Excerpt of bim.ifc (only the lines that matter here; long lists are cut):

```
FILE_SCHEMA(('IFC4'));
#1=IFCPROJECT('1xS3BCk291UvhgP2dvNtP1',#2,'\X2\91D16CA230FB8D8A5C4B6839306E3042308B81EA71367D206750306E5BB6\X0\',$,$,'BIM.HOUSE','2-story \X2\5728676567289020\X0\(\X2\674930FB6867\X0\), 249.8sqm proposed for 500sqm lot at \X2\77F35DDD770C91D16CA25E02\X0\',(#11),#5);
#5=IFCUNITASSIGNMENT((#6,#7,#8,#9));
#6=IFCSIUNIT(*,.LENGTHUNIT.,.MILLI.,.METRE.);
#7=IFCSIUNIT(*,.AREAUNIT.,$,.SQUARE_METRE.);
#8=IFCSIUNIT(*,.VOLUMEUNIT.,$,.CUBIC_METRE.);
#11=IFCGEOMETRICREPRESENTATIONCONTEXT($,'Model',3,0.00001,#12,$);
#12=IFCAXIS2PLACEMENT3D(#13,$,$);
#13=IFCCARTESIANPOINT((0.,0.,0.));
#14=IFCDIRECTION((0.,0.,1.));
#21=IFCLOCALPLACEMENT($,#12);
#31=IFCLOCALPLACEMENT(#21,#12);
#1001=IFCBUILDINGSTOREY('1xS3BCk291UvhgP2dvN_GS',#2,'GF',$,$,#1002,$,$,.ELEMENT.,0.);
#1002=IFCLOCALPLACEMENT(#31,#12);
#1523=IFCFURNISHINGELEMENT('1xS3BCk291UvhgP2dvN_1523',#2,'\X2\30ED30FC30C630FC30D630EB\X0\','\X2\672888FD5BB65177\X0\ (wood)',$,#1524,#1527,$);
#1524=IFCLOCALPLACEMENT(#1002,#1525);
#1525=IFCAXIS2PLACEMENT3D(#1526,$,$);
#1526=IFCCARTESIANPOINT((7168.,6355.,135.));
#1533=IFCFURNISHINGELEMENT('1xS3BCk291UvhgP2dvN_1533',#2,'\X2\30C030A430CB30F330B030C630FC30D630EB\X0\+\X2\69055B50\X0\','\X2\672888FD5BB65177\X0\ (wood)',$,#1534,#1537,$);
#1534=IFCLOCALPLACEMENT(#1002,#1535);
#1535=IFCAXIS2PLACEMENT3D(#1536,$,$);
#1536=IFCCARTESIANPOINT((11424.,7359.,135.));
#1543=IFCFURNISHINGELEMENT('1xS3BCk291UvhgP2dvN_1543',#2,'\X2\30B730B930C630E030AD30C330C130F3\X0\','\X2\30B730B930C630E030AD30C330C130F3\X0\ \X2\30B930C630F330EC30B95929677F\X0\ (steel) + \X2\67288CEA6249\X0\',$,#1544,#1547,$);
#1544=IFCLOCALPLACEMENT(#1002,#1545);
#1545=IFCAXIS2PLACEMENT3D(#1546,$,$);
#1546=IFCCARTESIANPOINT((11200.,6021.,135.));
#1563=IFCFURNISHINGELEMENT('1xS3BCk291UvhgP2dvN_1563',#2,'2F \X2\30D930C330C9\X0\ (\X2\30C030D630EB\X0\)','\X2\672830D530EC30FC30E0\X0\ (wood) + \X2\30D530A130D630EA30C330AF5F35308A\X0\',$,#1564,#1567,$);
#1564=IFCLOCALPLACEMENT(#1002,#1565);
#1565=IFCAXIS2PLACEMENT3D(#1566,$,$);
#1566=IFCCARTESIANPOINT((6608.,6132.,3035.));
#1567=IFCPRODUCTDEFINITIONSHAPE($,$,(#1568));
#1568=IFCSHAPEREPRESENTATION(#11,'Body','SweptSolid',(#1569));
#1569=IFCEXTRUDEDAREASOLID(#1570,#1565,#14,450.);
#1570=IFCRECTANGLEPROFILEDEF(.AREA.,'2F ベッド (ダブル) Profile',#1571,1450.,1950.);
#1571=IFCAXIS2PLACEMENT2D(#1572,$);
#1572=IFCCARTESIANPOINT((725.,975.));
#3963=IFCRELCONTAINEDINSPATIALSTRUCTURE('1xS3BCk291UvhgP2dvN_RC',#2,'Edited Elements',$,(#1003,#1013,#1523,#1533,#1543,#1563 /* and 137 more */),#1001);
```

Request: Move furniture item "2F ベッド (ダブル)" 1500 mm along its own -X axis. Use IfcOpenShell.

```python
import ifcopenshell
import ifcopenshell.api.geometry
import ifcopenshell.util.placement
import ifcopenshell.util.unit

model = ifcopenshell.open("bim.ifc")
unit_scale = ifcopenshell.util.unit.calculate_unit_scale(model)

item = model.by_guid("1xS3BCk291UvhgP2dvN_1563")
matrix = ifcopenshell.util.placement.get_local_placement(item.ObjectPlacement)
matrix[:3, 3] -= matrix[:3, 0] * 1.5 / unit_scale
ifcopenshell.api.geometry.edit_object_placement(model, product=item, matrix=matrix, is_si=False)

print(ifcopenshell.util.placement.get_local_placement(item.ObjectPlacement).round(3) + 0.0)

model.write("bim_v2.ifc")
```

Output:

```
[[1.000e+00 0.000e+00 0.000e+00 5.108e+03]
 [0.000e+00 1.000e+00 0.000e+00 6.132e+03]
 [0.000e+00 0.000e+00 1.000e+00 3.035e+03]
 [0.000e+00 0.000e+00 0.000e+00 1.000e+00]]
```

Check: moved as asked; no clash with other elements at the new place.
